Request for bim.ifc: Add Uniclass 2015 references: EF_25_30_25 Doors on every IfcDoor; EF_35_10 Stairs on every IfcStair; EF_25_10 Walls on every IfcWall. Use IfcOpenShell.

First a look at what the model holds.

```python
import ifcopenshell

model = ifcopenshell.open("bim.ifc")
print(model.schema)
print("classifications:", [c.Name for c in model.by_type("IfcClassification")])
for ifc_class in ("IfcDoor", "IfcRoof", "IfcStair", "IfcWall", "IfcWindow"):
    print(ifc_class, len(model.by_type(ifc_class)))
```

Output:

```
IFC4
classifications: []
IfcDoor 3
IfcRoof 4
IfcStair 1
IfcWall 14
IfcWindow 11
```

```python
import ifcopenshell
import ifcopenshell.api.classification

model = ifcopenshell.open("bim.ifc")

system = ifcopenshell.api.classification.add_classification(model, classification="Uniclass 2015")

codes = {
    "IfcDoor": ("EF_25_30_25", "Doors"),
    "IfcStair": ("EF_35_10", "Stairs"),
    "IfcWall": ("EF_25_10", "Walls"),
}
for ifc_class, (code, name) in codes.items():
    products = model.by_type(ifc_class)
    ifcopenshell.api.classification.add_reference(
        model, products=products, classification=system, identification=code, name=name
    )
    print(code, len(products))

model.write("bim_v2.ifc")
```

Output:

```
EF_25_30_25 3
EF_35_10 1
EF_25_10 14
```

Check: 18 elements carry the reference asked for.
